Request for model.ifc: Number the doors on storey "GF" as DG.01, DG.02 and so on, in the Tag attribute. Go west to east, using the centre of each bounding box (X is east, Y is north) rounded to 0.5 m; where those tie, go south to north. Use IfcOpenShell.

First a look at what the model holds.

```python
import ifcopenshell
import ifcopenshell.util.element
import ifcopenshell.util.placement

model = ifcopenshell.open("model.ifc")
print(model.schema)
storey = next(s for s in model.by_type("IfcBuildingStorey") if s.Name == "GF")
doors = [e for e in ifcopenshell.util.element.get_decomposition(storey) if e.is_a("IfcDoor")]
for e in sorted(doors, key=lambda e: e.id()):
    origin = ifcopenshell.util.placement.get_local_placement(e.ObjectPlacement)[:3, 3]
    print(e.id(), e.Tag, e.Name, origin.round(2) + 0.0, sep=" | ")
```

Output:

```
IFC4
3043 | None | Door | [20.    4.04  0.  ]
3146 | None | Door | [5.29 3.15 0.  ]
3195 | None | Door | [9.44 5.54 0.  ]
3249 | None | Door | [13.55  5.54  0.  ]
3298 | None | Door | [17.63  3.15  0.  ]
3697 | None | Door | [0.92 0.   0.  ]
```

```python
import ifcopenshell
import ifcopenshell.geom
import ifcopenshell.util.element
import ifcopenshell.util.shape

model = ifcopenshell.open("model.ifc")
settings = ifcopenshell.geom.settings()
settings.set("use-world-coords", True)


def centre(element):
    shape = ifcopenshell.geom.create_shape(settings, element)
    return ifcopenshell.util.shape.get_bbox_centroid(shape.geometry)


storey = next(s for s in model.by_type("IfcBuildingStorey") if s.Name == "GF")
doors = [e for e in ifcopenshell.util.element.get_decomposition(storey) if e.is_a("IfcDoor")]

# Insertion points can sit at a corner or the storey origin, so sort by the geometry (in metres).
centres = {e: centre(e) for e in doors}
doors.sort(key=lambda e: (round(centres[e][0] / 0.5), centres[e][1]))

for i, e in enumerate(doors, start=1):
    number = f"DG.{i:02d}"
    e.Tag = number
    print(e.id(), number)

model.write("model_updated.ifc")
```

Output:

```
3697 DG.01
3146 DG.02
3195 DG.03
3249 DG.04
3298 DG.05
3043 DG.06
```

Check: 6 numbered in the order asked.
